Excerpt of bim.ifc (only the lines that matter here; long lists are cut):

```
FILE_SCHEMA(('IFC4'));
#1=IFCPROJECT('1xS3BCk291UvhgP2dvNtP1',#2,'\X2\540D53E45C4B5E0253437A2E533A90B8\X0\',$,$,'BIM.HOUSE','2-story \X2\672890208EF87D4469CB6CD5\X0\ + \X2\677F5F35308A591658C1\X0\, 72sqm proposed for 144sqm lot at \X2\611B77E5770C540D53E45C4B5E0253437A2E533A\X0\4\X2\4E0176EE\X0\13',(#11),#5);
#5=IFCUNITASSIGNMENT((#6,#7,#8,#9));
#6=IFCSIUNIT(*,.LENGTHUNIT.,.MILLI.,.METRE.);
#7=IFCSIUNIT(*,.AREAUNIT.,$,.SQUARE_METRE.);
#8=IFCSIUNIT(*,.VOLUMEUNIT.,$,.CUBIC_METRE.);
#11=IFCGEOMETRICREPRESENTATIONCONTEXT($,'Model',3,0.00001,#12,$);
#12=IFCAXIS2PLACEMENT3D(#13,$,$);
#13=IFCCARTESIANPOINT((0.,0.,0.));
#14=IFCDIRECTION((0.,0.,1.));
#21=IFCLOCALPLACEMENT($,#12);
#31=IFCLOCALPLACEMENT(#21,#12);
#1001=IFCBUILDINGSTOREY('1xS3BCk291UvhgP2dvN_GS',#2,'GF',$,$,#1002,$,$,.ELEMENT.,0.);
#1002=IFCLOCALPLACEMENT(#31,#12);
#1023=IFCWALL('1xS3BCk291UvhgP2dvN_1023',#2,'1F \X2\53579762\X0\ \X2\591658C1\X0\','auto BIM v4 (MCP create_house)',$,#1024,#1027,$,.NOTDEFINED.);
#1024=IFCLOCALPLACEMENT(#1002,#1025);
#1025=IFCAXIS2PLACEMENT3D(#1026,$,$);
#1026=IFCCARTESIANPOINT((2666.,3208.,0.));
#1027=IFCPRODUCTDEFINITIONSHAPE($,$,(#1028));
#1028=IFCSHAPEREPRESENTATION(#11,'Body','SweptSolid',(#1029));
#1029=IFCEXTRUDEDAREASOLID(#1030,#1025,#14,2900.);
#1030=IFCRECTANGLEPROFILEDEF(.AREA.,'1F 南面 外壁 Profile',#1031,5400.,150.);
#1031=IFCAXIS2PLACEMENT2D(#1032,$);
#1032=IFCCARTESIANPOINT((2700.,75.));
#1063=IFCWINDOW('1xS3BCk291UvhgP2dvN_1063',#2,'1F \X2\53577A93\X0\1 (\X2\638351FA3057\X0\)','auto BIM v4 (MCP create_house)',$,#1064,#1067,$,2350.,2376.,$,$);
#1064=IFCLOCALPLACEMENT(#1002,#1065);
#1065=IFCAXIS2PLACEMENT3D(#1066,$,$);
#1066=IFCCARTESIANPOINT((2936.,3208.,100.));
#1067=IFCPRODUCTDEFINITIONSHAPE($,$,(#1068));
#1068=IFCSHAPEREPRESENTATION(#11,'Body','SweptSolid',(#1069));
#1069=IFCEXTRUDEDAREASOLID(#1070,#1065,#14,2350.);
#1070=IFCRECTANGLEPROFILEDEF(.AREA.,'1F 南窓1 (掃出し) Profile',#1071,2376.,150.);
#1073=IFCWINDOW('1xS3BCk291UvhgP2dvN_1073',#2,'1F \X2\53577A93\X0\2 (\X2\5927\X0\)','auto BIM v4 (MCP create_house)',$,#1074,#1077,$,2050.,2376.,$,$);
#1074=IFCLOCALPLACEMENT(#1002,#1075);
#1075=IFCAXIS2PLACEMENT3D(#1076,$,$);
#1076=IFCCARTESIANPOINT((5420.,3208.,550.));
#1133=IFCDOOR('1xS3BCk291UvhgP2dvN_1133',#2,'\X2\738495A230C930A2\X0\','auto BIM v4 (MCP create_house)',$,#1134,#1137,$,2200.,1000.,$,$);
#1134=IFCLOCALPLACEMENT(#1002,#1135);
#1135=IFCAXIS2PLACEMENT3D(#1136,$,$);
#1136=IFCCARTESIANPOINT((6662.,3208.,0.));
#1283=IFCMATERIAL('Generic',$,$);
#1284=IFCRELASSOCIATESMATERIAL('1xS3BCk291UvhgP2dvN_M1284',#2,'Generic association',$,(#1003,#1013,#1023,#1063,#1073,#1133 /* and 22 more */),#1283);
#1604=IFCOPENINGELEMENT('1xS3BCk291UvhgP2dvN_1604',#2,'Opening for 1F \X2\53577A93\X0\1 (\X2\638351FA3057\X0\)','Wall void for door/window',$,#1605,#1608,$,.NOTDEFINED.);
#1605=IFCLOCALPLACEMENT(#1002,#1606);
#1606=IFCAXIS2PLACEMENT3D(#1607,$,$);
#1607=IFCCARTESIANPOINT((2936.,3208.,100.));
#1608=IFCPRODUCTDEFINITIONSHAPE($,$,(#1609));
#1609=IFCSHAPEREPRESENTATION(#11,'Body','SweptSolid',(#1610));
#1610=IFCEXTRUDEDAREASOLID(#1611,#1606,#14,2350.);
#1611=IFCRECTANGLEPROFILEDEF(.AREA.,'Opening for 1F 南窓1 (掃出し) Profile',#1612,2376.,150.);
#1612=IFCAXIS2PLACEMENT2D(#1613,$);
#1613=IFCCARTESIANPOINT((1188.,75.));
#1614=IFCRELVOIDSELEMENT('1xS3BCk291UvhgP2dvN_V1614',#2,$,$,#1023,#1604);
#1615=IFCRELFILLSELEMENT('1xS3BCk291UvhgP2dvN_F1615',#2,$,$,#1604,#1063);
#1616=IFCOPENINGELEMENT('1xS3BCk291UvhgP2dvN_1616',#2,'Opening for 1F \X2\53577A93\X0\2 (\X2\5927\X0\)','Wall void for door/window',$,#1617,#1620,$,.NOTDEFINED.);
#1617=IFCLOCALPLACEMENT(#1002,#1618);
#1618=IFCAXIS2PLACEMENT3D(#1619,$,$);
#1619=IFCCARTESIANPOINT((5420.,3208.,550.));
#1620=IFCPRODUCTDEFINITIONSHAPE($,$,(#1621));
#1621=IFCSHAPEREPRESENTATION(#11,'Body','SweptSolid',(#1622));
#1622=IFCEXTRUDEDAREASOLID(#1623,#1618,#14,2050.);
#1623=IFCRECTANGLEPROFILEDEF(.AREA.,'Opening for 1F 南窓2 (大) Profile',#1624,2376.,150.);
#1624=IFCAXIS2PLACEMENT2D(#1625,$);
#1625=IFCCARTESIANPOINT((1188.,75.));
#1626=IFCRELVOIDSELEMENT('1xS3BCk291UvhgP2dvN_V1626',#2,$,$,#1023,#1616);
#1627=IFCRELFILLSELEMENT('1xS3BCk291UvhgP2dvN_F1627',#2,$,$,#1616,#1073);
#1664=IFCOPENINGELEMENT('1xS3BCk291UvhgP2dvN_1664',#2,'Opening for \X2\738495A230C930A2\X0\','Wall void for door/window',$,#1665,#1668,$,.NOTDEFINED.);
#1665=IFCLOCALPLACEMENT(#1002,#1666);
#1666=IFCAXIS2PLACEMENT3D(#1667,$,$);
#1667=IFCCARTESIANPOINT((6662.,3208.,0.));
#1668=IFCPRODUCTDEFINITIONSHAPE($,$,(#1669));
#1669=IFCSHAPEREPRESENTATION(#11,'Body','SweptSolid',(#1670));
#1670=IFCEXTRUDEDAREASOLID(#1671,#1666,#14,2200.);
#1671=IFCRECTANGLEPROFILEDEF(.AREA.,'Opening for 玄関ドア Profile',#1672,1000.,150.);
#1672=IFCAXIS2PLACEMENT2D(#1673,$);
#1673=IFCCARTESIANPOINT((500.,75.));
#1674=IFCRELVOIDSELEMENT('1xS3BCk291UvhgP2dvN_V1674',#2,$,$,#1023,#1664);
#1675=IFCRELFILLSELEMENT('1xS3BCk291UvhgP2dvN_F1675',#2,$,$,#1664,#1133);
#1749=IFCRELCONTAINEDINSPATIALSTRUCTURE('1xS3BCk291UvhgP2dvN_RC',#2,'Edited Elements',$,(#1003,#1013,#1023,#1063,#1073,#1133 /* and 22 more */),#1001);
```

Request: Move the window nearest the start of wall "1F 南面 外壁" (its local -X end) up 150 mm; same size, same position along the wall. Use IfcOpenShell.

```python
import numpy as np
import ifcopenshell
import ifcopenshell.api.geometry
import ifcopenshell.util.placement
import ifcopenshell.util.unit

model = ifcopenshell.open("bim.ifc")
unit_scale = ifcopenshell.util.unit.calculate_unit_scale(model)

window = model.by_guid("1xS3BCk291UvhgP2dvN_1063")
opening = window.FillsVoids[0].RelatingOpeningElement
dz = 0.15 / unit_scale

shift = np.array([0.0, 0.0, dz])
# The window is not placed relative to its opening, so move both.
for product in (opening, window):
    matrix = ifcopenshell.util.placement.get_local_placement(product.ObjectPlacement)
    matrix[:3, 3] += shift
    ifcopenshell.api.geometry.edit_object_placement(model, product=product, matrix=matrix, is_si=False)

print(f"moved by {dz * unit_scale:+.3f} m")

model.write("bim_updated.ifc")
```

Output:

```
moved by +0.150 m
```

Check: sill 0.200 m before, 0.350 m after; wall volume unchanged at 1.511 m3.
